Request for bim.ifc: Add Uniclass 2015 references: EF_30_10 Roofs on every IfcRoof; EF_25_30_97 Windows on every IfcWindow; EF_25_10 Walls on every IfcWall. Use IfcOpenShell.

First a look at what the model holds.

```python
import ifcopenshell

model = ifcopenshell.open("bim.ifc")
print(model.schema)
print("classifications:", [c.Name for c in model.by_type("IfcClassification")])
for ifc_class in ("IfcDoor", "IfcRoof", "IfcStair", "IfcWall", "IfcWindow"):
    print(ifc_class, len(model.by_type(ifc_class)))
```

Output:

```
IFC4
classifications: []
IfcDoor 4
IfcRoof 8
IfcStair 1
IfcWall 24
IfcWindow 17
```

```python
import ifcopenshell
import ifcopenshell.api.classification

model = ifcopenshell.open("bim.ifc")

system = ifcopenshell.api.classification.add_classification(model, classification="Uniclass 2015")

codes = {
    "IfcRoof": ("EF_30_10", "Roofs"),
    "IfcWindow": ("EF_25_30_97", "Windows"),
    "IfcWall": ("EF_25_10", "Walls"),
}
for ifc_class, (code, name) in codes.items():
    products = model.by_type(ifc_class)
    ifcopenshell.api.classification.add_reference(
        model, products=products, classification=system, identification=code, name=name
    )
    print(code, len(products))

model.write("bim-out.ifc")
```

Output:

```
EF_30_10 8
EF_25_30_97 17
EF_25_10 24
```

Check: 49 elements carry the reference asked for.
